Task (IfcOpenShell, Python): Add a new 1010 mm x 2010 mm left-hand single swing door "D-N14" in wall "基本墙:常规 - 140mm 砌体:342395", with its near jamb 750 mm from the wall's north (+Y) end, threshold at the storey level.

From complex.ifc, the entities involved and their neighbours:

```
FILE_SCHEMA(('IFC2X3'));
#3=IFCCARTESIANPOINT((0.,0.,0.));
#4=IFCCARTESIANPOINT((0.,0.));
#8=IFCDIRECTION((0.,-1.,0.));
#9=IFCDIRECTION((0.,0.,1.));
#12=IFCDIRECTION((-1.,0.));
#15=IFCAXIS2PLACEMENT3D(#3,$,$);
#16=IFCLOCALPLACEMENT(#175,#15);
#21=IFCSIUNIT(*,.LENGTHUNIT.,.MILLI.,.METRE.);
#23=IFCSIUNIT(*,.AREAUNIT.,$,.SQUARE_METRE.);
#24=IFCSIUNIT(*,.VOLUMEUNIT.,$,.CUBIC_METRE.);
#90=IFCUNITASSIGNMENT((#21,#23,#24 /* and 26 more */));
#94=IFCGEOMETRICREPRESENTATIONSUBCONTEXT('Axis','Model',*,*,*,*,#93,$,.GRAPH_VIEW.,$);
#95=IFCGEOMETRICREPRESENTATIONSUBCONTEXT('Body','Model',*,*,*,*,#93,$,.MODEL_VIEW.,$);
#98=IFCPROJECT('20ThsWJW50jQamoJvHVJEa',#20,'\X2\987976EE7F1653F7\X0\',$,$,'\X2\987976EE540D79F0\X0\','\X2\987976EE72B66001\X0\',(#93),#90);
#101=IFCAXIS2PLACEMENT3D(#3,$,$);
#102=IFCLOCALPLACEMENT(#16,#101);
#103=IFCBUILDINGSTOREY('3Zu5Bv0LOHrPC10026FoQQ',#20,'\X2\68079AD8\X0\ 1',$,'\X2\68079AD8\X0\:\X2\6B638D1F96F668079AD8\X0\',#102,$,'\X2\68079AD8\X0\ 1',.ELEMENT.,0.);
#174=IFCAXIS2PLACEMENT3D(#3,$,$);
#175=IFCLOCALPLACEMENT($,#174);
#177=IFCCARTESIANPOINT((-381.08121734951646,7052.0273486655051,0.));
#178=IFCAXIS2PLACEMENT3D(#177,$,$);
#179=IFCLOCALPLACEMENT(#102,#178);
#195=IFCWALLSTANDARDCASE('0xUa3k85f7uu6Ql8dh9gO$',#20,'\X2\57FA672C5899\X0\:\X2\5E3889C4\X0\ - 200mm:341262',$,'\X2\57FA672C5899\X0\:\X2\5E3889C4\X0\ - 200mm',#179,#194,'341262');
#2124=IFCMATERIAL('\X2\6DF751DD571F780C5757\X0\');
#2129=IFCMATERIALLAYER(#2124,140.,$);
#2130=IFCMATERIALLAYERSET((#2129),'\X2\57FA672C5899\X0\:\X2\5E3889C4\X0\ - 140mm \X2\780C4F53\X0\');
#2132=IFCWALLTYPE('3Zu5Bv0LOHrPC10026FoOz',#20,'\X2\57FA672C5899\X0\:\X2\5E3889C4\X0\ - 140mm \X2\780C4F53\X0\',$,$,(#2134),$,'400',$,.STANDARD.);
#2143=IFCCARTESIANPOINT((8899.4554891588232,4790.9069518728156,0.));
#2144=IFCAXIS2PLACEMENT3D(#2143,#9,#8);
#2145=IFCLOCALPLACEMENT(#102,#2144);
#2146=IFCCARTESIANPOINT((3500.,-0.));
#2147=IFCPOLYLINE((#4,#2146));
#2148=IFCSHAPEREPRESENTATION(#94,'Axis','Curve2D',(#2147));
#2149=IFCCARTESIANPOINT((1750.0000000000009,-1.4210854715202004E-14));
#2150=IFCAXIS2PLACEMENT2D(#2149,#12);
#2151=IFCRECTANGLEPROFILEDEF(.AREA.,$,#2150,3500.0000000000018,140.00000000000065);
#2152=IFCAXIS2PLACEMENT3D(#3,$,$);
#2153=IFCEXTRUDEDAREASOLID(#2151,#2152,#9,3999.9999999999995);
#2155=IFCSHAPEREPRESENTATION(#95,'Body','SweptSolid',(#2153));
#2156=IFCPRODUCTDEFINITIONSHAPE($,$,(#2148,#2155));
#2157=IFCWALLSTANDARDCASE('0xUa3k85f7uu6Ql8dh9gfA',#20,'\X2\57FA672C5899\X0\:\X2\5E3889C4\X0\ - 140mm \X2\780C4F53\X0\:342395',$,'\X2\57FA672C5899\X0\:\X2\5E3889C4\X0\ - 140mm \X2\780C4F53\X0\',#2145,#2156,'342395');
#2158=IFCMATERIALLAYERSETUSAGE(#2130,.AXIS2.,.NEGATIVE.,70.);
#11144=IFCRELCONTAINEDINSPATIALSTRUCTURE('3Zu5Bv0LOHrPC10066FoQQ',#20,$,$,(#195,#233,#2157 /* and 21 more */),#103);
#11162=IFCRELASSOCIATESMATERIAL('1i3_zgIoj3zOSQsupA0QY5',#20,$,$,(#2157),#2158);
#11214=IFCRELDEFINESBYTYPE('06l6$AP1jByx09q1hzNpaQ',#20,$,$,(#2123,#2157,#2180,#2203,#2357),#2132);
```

```python
import numpy as np
import ifcopenshell
import ifcopenshell.api.feature
import ifcopenshell.api.geometry
import ifcopenshell.api.root
import ifcopenshell.api.spatial
import ifcopenshell.api.type
import ifcopenshell.geom
import ifcopenshell.util.element
import ifcopenshell.util.placement
import ifcopenshell.util.representation
import ifcopenshell.util.shape
import ifcopenshell.util.unit

model = ifcopenshell.open("complex.ifc")
unit_scale = ifcopenshell.util.unit.calculate_unit_scale(model)
settings = ifcopenshell.geom.settings()


def volume(element):
    """Net volume in cubic metres, openings subtracted."""
    shape = ifcopenshell.geom.create_shape(settings, element)
    return ifcopenshell.util.shape.get_volume(shape.geometry)


wall = model.by_guid("0xUa3k85f7uu6Ql8dh9gfA")
storey = ifcopenshell.util.element.get_container(wall, ifc_class="IfcBuildingStorey")
context = ifcopenshell.util.representation.get_context(model, "Model", "Body", "MODEL_VIEW")
before = volume(wall)

width, height, from_end, sill = 1.01, 2.01, 0.75, 0.0  # metres

# The wall runs along its own X axis, and the end named is its -X end.
wall_shape = ifcopenshell.geom.create_shape(settings, wall)
x, y, z = ifcopenshell.util.shape.get_vertices(wall_shape.geometry).T
start = x.min() + from_end
face, thickness = float(y.min()), float(y.max() - y.min())
wall_matrix = ifcopenshell.util.placement.get_local_placement(wall.ObjectPlacement)
level = ifcopenshell.util.placement.get_local_placement(storey.ObjectPlacement)[2, 3]


def in_wall(x, y):
    """Placement at x, y metres in the wall's axes, at sill height."""
    matrix = wall_matrix.copy()
    matrix[:, 3] = wall_matrix @ np.array([x / unit_scale, y / unit_scale, 0.0, 1.0])
    matrix[2, 3] = level + sill / unit_scale
    return matrix


# Opening: a box that overshoots both wall faces by 50 mm.
opening = ifcopenshell.api.root.create_entity(model, ifc_class="IfcOpeningElement")
box = ifcopenshell.api.geometry.add_wall_representation(
    model, context=context, length=width, height=height, thickness=thickness + 0.1
)
ifcopenshell.api.geometry.assign_representation(model, product=opening, representation=box)
ifcopenshell.api.geometry.edit_object_placement(model, product=opening, matrix=in_wall(start, face - 0.05), is_si=False)
ifcopenshell.api.feature.add_feature(model, feature=opening, element=wall)

door = ifcopenshell.api.root.create_entity(model, ifc_class="IfcDoor", name="D-N14")
door.OverallWidth, door.OverallHeight = width / unit_scale, height / unit_scale
body = ifcopenshell.api.geometry.add_door_representation(
    model,
    context=context,
    overall_width=door.OverallWidth,
    overall_height=door.OverallHeight,
    operation_type="SINGLE_SWING_LEFT",
    lining_properties={"LiningDepth": thickness / unit_scale, "ThresholdDepth": thickness / unit_scale},
)
ifcopenshell.api.geometry.assign_representation(model, product=door, representation=body)
ifcopenshell.api.spatial.assign_container(model, products=[door], relating_structure=storey)
fills = ifcopenshell.api.feature.add_filling(model, opening=opening, element=door)
fills.OwnerHistory = door.OwnerHistory  # required in IFC2X3

# IFC2X3 keeps the operation on the door style.
style = ifcopenshell.api.root.create_entity(model, ifc_class="IfcDoorStyle", name="D-N14")
style.OperationType, style.ConstructionType = "SINGLE_SWING_LEFT", "NOTDEFINED"
style.ParameterTakesPrecedence = style.Sizeable = False
ifcopenshell.api.type.assign_type(model, related_objects=[door], relating_type=style)

# The lining spans the wall, so the door starts at the wall face.
ifcopenshell.api.geometry.edit_object_placement(model, product=door, matrix=in_wall(start, face), is_si=False)

after = volume(wall)

print(f"wall volume {before:.3f} -> {after:.3f} m3")

model.write("complex_rev.ifc")
```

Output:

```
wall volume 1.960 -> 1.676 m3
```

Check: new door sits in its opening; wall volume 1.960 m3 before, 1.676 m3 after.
